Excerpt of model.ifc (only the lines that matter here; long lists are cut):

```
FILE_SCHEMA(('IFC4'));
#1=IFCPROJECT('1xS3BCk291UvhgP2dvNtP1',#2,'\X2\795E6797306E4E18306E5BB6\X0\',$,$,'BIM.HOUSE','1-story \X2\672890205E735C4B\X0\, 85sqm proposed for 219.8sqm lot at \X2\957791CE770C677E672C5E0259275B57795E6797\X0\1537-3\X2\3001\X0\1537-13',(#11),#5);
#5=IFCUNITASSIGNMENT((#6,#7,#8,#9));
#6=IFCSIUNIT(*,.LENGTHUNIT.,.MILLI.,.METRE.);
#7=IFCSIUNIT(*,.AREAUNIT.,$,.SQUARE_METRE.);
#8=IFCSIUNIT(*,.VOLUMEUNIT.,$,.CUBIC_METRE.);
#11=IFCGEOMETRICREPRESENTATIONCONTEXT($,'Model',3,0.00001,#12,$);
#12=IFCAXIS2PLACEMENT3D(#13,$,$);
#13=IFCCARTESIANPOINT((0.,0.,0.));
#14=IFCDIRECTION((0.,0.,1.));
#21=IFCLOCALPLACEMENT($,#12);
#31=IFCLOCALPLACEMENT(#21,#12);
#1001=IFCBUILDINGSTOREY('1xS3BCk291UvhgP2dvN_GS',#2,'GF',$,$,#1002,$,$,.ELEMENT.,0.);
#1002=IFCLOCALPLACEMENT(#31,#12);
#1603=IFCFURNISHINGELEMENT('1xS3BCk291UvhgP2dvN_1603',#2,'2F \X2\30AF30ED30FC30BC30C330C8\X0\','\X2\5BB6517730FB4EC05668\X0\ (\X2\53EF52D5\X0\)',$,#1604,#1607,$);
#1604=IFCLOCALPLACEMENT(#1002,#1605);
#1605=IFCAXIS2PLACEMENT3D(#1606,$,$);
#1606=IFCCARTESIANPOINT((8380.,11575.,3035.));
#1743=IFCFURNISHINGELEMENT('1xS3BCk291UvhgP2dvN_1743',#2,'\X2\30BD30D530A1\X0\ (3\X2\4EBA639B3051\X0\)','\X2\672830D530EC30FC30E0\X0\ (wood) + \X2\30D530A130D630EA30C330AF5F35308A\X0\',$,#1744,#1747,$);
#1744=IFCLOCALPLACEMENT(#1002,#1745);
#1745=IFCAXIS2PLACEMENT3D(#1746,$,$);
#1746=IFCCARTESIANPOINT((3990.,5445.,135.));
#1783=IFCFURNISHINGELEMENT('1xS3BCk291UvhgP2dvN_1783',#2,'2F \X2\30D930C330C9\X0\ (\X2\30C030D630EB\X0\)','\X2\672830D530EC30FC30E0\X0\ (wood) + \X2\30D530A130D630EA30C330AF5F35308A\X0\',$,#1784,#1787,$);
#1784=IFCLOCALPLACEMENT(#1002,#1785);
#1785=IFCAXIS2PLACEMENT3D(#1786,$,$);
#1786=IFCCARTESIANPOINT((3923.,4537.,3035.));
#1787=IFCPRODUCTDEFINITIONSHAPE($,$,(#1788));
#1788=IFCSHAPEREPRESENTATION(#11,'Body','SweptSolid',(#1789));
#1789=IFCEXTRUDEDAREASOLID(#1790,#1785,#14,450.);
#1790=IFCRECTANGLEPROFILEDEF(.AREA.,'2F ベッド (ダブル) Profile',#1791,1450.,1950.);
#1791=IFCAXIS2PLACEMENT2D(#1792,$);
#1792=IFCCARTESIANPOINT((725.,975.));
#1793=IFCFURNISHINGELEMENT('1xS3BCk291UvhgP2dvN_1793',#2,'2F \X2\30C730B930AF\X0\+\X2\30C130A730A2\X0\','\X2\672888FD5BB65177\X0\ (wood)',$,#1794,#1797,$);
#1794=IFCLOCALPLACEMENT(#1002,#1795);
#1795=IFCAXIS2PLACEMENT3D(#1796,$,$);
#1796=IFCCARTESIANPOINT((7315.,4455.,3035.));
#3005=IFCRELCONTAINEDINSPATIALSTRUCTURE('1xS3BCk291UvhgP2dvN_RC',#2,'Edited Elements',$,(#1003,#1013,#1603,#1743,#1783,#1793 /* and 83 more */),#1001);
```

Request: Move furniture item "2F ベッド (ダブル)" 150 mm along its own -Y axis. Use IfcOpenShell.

```python
import ifcopenshell
import ifcopenshell.api.geometry
import ifcopenshell.util.placement
import ifcopenshell.util.unit

model = ifcopenshell.open("model.ifc")
unit_scale = ifcopenshell.util.unit.calculate_unit_scale(model)

item = model.by_id(1783)
matrix = ifcopenshell.util.placement.get_local_placement(item.ObjectPlacement)
matrix[:3, 3] -= matrix[:3, 1] * 0.15 / unit_scale
ifcopenshell.api.geometry.edit_object_placement(model, product=item, matrix=matrix, is_si=False)

print(ifcopenshell.util.placement.get_local_placement(item.ObjectPlacement).round(3) + 0.0)

model.write("model_v2.ifc")
```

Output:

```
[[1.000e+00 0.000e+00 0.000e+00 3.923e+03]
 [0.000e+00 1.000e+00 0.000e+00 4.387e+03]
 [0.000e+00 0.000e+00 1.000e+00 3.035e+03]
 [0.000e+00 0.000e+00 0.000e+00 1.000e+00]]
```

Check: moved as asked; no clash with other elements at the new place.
